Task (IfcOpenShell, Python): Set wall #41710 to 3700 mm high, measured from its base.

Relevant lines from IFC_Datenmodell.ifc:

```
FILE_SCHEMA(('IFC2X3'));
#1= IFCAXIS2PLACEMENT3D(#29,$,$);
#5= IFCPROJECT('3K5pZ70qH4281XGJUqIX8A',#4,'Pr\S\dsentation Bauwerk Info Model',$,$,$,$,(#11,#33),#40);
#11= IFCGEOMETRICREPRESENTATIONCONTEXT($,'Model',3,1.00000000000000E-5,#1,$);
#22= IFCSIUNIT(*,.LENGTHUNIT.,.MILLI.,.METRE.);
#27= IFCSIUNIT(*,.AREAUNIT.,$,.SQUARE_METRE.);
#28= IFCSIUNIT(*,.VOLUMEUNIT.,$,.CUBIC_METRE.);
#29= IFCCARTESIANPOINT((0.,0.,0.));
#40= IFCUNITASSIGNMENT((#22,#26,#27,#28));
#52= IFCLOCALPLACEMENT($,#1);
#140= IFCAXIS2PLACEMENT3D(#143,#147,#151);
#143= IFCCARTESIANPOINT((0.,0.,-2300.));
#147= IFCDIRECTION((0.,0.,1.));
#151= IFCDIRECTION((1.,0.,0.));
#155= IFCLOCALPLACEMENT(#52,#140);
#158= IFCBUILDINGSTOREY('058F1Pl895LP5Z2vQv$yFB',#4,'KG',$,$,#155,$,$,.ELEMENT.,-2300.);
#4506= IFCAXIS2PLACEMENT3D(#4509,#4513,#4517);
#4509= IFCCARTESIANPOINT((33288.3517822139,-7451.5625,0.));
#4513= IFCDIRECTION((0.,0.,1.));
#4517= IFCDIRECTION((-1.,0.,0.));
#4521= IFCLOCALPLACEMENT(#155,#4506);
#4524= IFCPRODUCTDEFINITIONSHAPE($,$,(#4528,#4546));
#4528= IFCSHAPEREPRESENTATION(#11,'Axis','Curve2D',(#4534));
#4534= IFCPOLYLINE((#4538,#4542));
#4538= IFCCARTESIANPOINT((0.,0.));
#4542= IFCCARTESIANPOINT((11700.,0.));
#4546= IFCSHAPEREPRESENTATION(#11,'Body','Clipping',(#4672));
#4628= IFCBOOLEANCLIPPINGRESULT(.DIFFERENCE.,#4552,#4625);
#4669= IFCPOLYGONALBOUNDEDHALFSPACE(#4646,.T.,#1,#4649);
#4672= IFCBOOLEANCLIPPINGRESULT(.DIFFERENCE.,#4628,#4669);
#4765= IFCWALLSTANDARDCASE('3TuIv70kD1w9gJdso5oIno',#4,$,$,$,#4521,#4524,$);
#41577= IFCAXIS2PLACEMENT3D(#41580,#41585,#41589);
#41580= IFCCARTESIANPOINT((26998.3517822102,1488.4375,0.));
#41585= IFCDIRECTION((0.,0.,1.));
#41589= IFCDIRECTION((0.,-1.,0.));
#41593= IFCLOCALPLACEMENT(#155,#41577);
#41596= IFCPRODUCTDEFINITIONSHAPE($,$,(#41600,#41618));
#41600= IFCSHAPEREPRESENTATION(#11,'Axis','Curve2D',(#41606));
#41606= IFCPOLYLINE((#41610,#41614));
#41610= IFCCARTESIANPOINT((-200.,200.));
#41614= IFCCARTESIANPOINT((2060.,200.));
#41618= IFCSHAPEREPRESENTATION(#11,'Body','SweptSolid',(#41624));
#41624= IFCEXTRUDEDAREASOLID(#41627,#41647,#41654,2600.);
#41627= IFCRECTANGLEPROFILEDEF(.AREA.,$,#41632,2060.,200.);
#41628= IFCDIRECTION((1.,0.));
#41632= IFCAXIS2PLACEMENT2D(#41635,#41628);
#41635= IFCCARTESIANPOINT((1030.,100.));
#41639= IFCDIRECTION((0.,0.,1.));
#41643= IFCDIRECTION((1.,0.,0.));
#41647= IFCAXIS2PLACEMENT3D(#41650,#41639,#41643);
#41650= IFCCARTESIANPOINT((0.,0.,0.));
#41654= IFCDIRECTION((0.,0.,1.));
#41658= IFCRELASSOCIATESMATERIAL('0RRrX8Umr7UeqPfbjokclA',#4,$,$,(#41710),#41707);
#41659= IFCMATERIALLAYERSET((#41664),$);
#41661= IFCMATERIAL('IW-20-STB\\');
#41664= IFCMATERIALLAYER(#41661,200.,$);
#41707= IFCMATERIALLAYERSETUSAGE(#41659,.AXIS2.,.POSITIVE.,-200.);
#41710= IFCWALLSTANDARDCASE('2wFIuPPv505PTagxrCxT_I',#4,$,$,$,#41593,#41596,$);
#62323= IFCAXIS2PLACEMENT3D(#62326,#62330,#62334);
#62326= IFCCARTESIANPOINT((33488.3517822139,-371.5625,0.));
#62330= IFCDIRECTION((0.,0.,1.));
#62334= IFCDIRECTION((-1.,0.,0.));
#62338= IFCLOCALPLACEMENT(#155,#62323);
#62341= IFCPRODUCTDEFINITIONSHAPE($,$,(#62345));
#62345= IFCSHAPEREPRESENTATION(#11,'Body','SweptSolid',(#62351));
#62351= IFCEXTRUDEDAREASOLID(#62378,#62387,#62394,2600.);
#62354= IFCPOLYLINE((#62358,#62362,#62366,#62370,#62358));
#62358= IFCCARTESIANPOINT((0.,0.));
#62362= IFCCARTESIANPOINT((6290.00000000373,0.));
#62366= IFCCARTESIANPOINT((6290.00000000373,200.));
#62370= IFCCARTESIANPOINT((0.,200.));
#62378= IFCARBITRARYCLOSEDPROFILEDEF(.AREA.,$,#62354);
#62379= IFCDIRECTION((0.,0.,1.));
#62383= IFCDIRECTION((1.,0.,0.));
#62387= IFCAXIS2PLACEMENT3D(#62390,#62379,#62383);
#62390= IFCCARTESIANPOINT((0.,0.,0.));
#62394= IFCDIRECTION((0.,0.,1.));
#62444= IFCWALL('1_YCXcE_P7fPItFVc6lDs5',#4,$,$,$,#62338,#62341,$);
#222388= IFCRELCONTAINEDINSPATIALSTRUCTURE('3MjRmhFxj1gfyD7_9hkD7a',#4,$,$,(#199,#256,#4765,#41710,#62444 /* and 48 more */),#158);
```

```python
import ifcopenshell
import ifcopenshell.geom
import ifcopenshell.util.shape
import ifcopenshell.util.unit

model = ifcopenshell.open("IFC_Datenmodell.ifc")
unit_scale = ifcopenshell.util.unit.calculate_unit_scale(model)
settings = ifcopenshell.geom.settings()


def volume(element):
    """Net volume in cubic metres, openings subtracted."""
    shape = ifcopenshell.geom.create_shape(settings, element)
    return ifcopenshell.util.shape.get_volume(shape.geometry)


wall = model.by_id(41710)
before = volume(wall)

body = next(r for r in wall.Representation.Representations if r.RepresentationIdentifier == "Body")
solid = body.Items[0]
old_height = solid.Depth
solid.Depth = 3.7 / unit_scale
after = volume(wall)

print(f"height {old_height:g} -> {solid.Depth:g}, volume {before:.3f} -> {after:.3f} m3")

model.write("IFC_Datenmodell_edited.ifc")
```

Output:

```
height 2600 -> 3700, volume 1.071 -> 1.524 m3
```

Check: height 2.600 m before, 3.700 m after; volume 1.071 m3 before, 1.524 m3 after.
